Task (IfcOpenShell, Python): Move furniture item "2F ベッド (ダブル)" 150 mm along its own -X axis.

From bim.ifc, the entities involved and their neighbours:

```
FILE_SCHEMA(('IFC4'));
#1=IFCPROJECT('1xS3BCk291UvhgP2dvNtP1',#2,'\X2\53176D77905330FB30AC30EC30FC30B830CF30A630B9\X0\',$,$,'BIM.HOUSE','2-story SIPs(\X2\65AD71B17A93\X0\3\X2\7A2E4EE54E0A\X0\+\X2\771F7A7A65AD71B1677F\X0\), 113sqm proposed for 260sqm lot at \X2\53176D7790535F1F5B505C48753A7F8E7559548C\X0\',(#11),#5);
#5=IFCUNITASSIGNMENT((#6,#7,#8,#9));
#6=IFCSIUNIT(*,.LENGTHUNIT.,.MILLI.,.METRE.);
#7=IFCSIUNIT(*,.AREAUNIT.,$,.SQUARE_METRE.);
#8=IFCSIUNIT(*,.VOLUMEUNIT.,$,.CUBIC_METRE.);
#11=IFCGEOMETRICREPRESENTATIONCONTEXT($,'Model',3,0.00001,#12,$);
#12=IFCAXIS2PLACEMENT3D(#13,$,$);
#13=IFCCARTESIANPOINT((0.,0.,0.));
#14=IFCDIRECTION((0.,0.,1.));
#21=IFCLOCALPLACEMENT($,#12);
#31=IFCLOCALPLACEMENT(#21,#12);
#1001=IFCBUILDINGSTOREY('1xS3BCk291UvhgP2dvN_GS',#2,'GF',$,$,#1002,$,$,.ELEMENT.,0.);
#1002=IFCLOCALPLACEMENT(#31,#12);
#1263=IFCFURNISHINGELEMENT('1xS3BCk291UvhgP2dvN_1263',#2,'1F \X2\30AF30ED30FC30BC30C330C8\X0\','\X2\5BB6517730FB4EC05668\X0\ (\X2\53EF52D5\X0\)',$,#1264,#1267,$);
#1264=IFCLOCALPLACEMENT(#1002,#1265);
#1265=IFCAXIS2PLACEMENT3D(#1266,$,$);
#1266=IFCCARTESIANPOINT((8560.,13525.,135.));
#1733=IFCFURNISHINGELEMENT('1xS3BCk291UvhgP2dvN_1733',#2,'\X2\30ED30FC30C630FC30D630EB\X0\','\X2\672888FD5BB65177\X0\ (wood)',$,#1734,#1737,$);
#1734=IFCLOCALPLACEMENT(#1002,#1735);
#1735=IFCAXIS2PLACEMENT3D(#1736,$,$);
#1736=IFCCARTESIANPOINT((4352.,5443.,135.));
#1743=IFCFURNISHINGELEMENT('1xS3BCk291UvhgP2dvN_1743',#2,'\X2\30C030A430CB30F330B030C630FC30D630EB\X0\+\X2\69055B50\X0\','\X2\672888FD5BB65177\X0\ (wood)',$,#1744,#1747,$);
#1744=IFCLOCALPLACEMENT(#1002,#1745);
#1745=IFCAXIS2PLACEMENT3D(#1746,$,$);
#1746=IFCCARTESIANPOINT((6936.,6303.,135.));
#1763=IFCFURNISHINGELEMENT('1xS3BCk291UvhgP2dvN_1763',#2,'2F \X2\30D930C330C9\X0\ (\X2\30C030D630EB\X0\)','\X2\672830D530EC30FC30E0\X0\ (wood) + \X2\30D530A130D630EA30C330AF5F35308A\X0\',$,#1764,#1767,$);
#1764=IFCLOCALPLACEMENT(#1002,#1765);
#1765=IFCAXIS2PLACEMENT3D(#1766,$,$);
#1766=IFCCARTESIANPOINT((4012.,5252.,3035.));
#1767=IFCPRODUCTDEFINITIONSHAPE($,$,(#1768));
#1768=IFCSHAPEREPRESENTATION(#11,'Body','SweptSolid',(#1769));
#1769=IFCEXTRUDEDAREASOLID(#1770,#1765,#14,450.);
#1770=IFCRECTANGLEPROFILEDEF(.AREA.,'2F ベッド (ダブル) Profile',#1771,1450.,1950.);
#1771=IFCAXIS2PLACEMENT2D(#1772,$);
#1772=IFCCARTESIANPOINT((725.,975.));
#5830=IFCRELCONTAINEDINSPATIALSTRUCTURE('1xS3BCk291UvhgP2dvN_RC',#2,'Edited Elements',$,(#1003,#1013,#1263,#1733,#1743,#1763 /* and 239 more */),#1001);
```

```python
import ifcopenshell
import ifcopenshell.api.geometry
import ifcopenshell.util.placement

model = ifcopenshell.open("bim.ifc")

item = model.by_id(1763)
matrix = ifcopenshell.util.placement.get_local_placement(item.ObjectPlacement)
matrix[:3, 3] -= matrix[:3, 0] * 150.0
ifcopenshell.api.geometry.edit_object_placement(model, product=item, matrix=matrix, is_si=False)

print(ifcopenshell.util.placement.get_local_placement(item.ObjectPlacement).round(3) + 0.0)

model.write("bim-out.ifc")
```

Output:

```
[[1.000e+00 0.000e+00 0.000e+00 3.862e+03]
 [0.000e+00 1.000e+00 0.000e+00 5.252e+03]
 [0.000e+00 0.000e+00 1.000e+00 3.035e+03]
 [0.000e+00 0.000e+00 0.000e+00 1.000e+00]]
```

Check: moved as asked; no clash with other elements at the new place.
